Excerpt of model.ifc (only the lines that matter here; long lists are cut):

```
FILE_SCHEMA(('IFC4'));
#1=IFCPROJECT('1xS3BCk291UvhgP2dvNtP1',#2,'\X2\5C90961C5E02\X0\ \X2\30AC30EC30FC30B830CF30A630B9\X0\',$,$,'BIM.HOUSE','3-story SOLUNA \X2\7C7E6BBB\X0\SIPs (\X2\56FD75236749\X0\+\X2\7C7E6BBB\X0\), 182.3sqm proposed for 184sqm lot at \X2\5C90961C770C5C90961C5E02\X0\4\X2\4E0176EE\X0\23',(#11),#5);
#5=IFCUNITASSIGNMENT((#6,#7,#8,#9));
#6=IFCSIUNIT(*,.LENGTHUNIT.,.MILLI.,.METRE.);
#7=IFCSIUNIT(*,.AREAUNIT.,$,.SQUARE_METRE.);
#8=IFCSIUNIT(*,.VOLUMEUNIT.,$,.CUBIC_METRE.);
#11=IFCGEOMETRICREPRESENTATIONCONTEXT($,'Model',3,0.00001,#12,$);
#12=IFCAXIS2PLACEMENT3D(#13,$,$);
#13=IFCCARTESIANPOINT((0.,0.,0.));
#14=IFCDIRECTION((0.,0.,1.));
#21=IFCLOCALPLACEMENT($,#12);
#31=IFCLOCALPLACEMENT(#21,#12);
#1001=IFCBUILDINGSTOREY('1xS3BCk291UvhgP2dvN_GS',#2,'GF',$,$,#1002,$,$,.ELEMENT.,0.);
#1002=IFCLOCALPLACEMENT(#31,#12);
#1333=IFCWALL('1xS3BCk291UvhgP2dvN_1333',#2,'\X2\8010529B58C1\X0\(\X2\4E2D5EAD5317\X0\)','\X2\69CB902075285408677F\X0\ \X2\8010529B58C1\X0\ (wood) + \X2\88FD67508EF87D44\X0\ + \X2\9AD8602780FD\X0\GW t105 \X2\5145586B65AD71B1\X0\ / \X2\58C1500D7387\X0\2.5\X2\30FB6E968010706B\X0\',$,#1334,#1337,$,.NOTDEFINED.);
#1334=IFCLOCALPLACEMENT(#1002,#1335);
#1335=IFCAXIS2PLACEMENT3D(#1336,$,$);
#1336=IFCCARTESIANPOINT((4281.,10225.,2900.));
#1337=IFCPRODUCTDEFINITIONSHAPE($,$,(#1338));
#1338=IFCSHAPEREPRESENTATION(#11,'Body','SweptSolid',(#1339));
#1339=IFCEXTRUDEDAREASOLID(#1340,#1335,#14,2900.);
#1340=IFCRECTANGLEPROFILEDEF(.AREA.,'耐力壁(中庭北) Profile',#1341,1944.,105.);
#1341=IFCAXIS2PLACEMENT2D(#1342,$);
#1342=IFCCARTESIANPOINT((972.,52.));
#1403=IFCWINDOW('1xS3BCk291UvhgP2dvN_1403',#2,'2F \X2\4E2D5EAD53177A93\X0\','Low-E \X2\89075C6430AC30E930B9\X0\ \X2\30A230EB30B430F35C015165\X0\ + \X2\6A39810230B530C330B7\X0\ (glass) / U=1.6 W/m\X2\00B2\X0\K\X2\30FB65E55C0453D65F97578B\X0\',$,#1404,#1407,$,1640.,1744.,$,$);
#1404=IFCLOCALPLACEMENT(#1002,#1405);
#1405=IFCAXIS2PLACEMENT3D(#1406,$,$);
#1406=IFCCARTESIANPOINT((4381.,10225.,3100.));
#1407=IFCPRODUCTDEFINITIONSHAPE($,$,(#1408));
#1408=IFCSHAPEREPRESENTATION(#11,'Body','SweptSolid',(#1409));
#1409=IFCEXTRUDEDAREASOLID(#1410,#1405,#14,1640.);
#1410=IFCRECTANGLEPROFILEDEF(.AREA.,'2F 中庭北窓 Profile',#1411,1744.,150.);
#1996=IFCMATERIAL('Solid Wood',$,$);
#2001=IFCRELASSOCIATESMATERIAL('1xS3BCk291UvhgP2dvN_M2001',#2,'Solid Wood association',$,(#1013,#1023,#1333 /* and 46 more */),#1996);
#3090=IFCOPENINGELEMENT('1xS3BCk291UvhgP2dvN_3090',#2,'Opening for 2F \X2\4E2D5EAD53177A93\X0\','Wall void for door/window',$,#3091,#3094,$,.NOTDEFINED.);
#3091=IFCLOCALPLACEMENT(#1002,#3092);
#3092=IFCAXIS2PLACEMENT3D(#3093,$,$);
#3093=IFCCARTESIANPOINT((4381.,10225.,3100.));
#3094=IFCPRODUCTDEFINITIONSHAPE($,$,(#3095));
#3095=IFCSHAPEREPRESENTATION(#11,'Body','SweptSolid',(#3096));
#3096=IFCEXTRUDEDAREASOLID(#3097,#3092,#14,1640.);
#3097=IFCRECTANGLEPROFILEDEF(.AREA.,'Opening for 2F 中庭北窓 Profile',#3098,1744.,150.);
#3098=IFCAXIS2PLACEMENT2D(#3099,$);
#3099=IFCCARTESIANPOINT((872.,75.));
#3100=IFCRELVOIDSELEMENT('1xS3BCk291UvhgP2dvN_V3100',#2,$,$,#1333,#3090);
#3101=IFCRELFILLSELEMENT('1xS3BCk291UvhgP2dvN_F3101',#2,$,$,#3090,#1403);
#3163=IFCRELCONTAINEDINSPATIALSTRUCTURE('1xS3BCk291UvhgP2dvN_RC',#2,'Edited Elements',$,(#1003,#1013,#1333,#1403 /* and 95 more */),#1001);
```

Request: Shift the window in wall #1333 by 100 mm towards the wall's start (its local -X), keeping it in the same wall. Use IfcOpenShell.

```python
import ifcopenshell
import ifcopenshell.api.geometry
import ifcopenshell.util.placement
import ifcopenshell.util.unit

model = ifcopenshell.open("model.ifc")
unit_scale = ifcopenshell.util.unit.calculate_unit_scale(model)

window = model.by_id(1403)
opening = window.FillsVoids[0].RelatingOpeningElement
wall = opening.VoidsElements[0].RelatingBuildingElement

wall_matrix = ifcopenshell.util.placement.get_local_placement(wall.ObjectPlacement)
shift = wall_matrix[:3, 0] * -0.1 / unit_scale
before = ifcopenshell.util.placement.get_local_placement(window.ObjectPlacement)[:3, 3].copy()

# The window is not placed relative to its opening, so move both.
for product in (opening, window):
    matrix = ifcopenshell.util.placement.get_local_placement(product.ObjectPlacement)
    matrix[:3, 3] += shift
    ifcopenshell.api.geometry.edit_object_placement(model, product=product, matrix=matrix, is_si=False)

after = ifcopenshell.util.placement.get_local_placement(window.ObjectPlacement)[:3, 3]
print("window moved by", (after - before).round(3) + 0.0)

model.write("model-out.ifc")
```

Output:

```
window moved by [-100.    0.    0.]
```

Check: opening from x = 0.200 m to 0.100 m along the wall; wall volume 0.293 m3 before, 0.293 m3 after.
